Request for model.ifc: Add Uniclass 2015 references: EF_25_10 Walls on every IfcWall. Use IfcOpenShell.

First a look at what the model holds.

```python
import ifcopenshell

model = ifcopenshell.open("model.ifc")
print(model.schema)
print("classifications:", [c.Name for c in model.by_type("IfcClassification")])
for ifc_class in ("IfcDoor", "IfcRoof", "IfcStair", "IfcWall", "IfcWindow"):
    print(ifc_class, len(model.by_type(ifc_class)))
```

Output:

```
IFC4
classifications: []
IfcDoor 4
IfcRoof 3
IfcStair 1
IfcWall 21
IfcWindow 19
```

```python
import ifcopenshell
import ifcopenshell.api.classification

model = ifcopenshell.open("model.ifc")

system = ifcopenshell.api.classification.add_classification(model, classification="Uniclass 2015")

codes = {
    "IfcWall": ("EF_25_10", "Walls"),
}
for ifc_class, (code, name) in codes.items():
    products = model.by_type(ifc_class)
    ifcopenshell.api.classification.add_reference(
        model, products=products, classification=system, identification=code, name=name
    )
    print(code, len(products))

model.write("model-out.ifc")
```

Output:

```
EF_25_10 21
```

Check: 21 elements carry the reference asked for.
